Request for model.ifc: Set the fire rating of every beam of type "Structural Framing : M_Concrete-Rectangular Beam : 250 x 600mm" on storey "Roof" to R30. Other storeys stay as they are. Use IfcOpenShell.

First a look at what the model holds.

```python
import ifcopenshell
import ifcopenshell.util.element

model = ifcopenshell.open("model.ifc")
print(model.schema)
storey = next(s for s in model.by_type("IfcBuildingStorey") if s.Name == "Roof")
beams = [e for e in ifcopenshell.util.element.get_decomposition(storey) if e.is_a("IfcBeam")]
seen = {}
for e in beams:
    element_type = ifcopenshell.util.element.get_type(e)
    key = (element_type.Name if element_type != e and element_type else None, ifcopenshell.util.element.get_pset(e, "Pset_BeamCommon", "FireRating"))
    seen[key] = seen.get(key, 0) + 1
for (name, value), count in sorted(seen.items(), key=str):
    print(count, "x", name, "|", value)
```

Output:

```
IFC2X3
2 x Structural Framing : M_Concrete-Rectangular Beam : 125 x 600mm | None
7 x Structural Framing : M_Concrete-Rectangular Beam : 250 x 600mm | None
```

```python
import ifcopenshell
import ifcopenshell.api.pset
import ifcopenshell.util.element

model = ifcopenshell.open("model.ifc")

storey = next(s for s in model.by_type("IfcBuildingStorey") if s.Name == "Roof")
beams = [e for e in ifcopenshell.util.element.get_decomposition(storey) if e.is_a("IfcBeam")]

count = 0
for e in beams:
    element_type = ifcopenshell.util.element.get_type(e)
    if element_type in (None, e) or element_type.Name != "Structural Framing : M_Concrete-Rectangular Beam : 250 x 600mm":
        continue
    # add_pset returns the element's existing set when there is one.
    pset = ifcopenshell.api.pset.add_pset(model, product=e, name="Pset_BeamCommon")
    ifcopenshell.api.pset.edit_pset(model, pset=pset, properties={"FireRating": "R30"})
    count += 1

print(count, "beams updated")

model.write("model_updated.ifc")
```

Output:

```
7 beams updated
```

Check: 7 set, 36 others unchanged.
